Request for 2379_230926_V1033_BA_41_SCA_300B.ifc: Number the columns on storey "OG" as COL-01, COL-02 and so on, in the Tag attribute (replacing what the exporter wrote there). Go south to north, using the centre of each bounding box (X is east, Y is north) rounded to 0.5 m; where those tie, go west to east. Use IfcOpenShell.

First a look at what the model holds.

```python
import ifcopenshell
import ifcopenshell.util.element
import ifcopenshell.util.placement

model = ifcopenshell.open("2379_230926_V1033_BA_41_SCA_300B.ifc")
print(model.schema)
storey = next(s for s in model.by_type("IfcBuildingStorey") if s.Name == "OG")
columns = [e for e in ifcopenshell.util.element.get_decomposition(storey) if e.is_a("IfcColumn")]
for e in sorted(columns, key=lambda e: e.id()):
    origin = ifcopenshell.util.placement.get_local_placement(e.ObjectPlacement)[:3, 3]
    print(e.id(), e.Tag, e.Name, origin.round(2) + 0.0, sep=" | ")
```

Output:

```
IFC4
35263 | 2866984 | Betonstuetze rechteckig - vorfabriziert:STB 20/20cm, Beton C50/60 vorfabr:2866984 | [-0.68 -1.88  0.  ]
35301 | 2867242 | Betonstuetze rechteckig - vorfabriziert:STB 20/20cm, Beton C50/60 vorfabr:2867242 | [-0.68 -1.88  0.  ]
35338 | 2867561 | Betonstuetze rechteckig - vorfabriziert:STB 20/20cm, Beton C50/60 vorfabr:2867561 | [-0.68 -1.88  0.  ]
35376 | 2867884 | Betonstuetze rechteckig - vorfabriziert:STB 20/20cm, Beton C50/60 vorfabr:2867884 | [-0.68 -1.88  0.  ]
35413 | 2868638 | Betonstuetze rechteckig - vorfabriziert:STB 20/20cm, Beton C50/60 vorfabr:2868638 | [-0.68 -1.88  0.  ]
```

```python
import ifcopenshell
import ifcopenshell.geom
import ifcopenshell.util.element
import ifcopenshell.util.shape

model = ifcopenshell.open("2379_230926_V1033_BA_41_SCA_300B.ifc")
settings = ifcopenshell.geom.settings()
settings.set("use-world-coords", True)


def centre(element):
    shape = ifcopenshell.geom.create_shape(settings, element)
    return ifcopenshell.util.shape.get_bbox_centroid(shape.geometry)


storey = next(s for s in model.by_type("IfcBuildingStorey") if s.Name == "OG")
columns = [e for e in ifcopenshell.util.element.get_decomposition(storey) if e.is_a("IfcColumn")]

# Insertion points can sit at a corner or the storey origin, so sort by the geometry (in metres).
centres = {e: centre(e) for e in columns}
columns.sort(key=lambda e: (round(centres[e][1] / 0.5), centres[e][0]))

for i, e in enumerate(columns, start=1):
    number = f"COL-{i:02d}"
    e.Tag = number
    print(e.id(), number)

model.write("2379_230926_V1033_BA_41_SCA_300B_v2.ifc")
```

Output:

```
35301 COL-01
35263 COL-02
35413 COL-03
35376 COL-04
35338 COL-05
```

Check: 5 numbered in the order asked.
